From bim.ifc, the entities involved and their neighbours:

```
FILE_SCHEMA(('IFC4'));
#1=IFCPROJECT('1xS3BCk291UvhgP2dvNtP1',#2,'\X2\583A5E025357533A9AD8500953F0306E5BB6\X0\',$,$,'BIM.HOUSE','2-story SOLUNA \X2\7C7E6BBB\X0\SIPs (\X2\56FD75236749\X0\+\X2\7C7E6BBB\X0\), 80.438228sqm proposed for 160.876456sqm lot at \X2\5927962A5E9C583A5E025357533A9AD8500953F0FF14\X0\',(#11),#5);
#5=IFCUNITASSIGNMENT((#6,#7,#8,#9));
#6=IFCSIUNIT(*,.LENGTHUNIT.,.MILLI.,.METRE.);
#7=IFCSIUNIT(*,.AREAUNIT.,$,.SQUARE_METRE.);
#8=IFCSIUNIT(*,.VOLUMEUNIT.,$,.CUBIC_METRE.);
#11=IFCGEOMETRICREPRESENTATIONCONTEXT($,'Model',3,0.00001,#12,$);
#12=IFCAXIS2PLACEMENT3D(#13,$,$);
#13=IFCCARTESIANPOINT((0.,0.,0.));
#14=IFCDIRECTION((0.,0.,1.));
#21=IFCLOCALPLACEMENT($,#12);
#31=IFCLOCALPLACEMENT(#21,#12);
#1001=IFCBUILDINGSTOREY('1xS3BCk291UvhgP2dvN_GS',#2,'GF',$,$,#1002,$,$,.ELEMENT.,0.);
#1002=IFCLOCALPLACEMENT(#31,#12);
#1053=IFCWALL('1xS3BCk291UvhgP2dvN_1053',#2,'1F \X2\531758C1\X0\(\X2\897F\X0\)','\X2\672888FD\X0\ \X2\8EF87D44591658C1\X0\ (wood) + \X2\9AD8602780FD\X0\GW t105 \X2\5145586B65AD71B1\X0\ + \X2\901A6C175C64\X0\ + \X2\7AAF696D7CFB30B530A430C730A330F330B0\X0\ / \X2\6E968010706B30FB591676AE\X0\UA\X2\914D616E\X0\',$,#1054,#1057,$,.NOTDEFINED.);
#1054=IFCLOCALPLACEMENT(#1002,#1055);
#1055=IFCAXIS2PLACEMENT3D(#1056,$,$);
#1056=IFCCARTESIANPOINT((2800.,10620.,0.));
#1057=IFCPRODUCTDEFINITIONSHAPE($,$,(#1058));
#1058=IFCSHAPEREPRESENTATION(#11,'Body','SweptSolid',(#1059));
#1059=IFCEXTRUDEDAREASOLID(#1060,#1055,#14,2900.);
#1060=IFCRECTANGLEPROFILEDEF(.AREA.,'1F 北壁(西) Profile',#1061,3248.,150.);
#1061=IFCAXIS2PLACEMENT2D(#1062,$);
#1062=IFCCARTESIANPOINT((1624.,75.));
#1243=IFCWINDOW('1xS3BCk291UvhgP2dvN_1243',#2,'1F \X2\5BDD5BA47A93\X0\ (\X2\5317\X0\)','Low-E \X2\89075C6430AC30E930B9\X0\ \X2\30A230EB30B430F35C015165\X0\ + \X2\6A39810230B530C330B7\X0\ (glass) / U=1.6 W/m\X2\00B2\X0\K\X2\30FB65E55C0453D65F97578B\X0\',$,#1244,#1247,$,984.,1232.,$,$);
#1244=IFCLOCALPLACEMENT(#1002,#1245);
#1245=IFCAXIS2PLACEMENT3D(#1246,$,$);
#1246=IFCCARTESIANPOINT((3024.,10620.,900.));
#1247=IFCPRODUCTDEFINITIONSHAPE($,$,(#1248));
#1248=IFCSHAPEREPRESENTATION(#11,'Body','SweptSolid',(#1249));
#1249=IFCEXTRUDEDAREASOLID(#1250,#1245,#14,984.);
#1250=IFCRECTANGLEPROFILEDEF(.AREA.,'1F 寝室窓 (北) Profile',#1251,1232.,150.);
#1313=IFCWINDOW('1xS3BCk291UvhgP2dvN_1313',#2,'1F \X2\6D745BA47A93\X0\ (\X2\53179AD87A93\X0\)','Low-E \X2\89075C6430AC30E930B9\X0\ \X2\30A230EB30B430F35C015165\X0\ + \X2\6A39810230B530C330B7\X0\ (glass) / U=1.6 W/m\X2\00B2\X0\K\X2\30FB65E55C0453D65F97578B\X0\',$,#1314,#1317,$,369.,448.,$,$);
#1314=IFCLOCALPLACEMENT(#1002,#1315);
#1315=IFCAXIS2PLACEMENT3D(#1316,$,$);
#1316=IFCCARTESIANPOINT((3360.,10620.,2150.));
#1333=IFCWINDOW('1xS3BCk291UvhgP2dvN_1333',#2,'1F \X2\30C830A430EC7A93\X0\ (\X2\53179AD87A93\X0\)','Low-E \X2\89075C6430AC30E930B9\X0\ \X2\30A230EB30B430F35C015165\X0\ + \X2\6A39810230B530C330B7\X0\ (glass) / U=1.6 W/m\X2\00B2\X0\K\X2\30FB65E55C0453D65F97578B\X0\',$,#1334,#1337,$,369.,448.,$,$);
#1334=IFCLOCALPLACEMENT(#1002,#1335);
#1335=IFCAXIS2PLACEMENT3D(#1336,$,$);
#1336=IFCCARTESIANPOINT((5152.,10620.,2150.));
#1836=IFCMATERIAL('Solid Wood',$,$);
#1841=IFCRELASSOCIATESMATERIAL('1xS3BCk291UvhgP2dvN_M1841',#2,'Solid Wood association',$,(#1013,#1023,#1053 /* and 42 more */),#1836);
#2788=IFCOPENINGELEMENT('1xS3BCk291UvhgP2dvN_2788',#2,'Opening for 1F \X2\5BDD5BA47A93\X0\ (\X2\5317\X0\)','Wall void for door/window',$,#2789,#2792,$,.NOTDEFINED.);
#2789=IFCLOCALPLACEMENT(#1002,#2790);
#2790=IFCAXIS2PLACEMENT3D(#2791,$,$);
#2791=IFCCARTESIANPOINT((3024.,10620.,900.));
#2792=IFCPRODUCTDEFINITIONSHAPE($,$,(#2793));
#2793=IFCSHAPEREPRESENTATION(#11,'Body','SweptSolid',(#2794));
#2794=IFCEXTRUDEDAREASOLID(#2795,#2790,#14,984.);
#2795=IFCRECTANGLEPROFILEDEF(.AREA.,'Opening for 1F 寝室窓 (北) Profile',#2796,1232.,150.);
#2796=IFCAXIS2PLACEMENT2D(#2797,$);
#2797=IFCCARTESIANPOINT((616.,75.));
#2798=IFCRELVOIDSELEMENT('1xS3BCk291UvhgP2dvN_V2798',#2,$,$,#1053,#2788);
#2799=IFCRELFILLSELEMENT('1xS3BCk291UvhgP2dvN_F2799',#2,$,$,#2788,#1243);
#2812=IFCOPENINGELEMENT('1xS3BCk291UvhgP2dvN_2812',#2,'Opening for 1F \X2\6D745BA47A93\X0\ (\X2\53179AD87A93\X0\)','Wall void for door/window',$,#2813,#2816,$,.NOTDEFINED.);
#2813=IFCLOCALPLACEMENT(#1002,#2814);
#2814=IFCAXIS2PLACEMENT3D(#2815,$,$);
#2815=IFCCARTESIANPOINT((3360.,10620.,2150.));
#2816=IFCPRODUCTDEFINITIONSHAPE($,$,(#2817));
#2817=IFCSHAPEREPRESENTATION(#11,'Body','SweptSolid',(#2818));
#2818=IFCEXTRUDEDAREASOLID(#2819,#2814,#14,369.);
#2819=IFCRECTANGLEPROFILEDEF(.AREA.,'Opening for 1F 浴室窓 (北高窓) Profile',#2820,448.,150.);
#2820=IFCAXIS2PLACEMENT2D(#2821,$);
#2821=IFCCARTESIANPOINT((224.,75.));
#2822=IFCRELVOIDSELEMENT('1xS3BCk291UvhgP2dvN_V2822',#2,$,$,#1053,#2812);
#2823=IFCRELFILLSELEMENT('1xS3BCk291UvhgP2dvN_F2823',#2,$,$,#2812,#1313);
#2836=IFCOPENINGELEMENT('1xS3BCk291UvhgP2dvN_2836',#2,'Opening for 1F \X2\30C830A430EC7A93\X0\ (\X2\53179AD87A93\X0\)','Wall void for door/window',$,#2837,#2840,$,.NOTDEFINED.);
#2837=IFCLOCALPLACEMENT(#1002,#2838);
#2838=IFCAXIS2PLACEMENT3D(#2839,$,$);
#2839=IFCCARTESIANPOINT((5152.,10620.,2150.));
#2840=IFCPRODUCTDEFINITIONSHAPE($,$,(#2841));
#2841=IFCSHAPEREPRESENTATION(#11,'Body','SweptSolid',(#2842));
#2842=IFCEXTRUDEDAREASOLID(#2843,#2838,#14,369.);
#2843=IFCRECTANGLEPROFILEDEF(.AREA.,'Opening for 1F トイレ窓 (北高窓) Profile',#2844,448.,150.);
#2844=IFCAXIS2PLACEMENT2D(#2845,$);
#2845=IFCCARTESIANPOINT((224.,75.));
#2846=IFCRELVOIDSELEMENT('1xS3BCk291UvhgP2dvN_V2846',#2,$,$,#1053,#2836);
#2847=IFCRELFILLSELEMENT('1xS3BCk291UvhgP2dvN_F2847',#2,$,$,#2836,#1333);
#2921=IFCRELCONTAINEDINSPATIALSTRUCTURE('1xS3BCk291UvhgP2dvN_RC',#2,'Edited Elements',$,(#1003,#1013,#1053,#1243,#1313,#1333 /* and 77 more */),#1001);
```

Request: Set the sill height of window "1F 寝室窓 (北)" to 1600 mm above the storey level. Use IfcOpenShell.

```python
import numpy as np
import ifcopenshell
import ifcopenshell.api.geometry
import ifcopenshell.geom
import ifcopenshell.util.element
import ifcopenshell.util.placement
import ifcopenshell.util.shape
import ifcopenshell.util.unit

model = ifcopenshell.open("bim.ifc")
unit_scale = ifcopenshell.util.unit.calculate_unit_scale(model)

window = model.by_guid("1xS3BCk291UvhgP2dvN_1243")
opening = window.FillsVoids[0].RelatingOpeningElement
storey = ifcopenshell.util.element.get_container(window, ifc_class="IfcBuildingStorey")
level = ifcopenshell.util.placement.get_local_placement(storey.ObjectPlacement)[2, 3]

# The opening's origin need not be at the sill, so measure its lowest point.
shape = ifcopenshell.geom.create_shape(ifcopenshell.geom.settings(), opening)
bottom = ifcopenshell.util.shape.get_shape_bottom_elevation(shape, shape.geometry) / unit_scale
dz = level + 1600.0 - bottom

shift = np.array([0.0, 0.0, dz])
# The window is not placed relative to its opening, so move both.
for product in (opening, window):
    matrix = ifcopenshell.util.placement.get_local_placement(product.ObjectPlacement)
    matrix[:3, 3] += shift
    ifcopenshell.api.geometry.edit_object_placement(model, product=product, matrix=matrix, is_si=False)

print(f"moved by {dz * unit_scale:+.3f} m")

model.write("bim-out.ifc")
```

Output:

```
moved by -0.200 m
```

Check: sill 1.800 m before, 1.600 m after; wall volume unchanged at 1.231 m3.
